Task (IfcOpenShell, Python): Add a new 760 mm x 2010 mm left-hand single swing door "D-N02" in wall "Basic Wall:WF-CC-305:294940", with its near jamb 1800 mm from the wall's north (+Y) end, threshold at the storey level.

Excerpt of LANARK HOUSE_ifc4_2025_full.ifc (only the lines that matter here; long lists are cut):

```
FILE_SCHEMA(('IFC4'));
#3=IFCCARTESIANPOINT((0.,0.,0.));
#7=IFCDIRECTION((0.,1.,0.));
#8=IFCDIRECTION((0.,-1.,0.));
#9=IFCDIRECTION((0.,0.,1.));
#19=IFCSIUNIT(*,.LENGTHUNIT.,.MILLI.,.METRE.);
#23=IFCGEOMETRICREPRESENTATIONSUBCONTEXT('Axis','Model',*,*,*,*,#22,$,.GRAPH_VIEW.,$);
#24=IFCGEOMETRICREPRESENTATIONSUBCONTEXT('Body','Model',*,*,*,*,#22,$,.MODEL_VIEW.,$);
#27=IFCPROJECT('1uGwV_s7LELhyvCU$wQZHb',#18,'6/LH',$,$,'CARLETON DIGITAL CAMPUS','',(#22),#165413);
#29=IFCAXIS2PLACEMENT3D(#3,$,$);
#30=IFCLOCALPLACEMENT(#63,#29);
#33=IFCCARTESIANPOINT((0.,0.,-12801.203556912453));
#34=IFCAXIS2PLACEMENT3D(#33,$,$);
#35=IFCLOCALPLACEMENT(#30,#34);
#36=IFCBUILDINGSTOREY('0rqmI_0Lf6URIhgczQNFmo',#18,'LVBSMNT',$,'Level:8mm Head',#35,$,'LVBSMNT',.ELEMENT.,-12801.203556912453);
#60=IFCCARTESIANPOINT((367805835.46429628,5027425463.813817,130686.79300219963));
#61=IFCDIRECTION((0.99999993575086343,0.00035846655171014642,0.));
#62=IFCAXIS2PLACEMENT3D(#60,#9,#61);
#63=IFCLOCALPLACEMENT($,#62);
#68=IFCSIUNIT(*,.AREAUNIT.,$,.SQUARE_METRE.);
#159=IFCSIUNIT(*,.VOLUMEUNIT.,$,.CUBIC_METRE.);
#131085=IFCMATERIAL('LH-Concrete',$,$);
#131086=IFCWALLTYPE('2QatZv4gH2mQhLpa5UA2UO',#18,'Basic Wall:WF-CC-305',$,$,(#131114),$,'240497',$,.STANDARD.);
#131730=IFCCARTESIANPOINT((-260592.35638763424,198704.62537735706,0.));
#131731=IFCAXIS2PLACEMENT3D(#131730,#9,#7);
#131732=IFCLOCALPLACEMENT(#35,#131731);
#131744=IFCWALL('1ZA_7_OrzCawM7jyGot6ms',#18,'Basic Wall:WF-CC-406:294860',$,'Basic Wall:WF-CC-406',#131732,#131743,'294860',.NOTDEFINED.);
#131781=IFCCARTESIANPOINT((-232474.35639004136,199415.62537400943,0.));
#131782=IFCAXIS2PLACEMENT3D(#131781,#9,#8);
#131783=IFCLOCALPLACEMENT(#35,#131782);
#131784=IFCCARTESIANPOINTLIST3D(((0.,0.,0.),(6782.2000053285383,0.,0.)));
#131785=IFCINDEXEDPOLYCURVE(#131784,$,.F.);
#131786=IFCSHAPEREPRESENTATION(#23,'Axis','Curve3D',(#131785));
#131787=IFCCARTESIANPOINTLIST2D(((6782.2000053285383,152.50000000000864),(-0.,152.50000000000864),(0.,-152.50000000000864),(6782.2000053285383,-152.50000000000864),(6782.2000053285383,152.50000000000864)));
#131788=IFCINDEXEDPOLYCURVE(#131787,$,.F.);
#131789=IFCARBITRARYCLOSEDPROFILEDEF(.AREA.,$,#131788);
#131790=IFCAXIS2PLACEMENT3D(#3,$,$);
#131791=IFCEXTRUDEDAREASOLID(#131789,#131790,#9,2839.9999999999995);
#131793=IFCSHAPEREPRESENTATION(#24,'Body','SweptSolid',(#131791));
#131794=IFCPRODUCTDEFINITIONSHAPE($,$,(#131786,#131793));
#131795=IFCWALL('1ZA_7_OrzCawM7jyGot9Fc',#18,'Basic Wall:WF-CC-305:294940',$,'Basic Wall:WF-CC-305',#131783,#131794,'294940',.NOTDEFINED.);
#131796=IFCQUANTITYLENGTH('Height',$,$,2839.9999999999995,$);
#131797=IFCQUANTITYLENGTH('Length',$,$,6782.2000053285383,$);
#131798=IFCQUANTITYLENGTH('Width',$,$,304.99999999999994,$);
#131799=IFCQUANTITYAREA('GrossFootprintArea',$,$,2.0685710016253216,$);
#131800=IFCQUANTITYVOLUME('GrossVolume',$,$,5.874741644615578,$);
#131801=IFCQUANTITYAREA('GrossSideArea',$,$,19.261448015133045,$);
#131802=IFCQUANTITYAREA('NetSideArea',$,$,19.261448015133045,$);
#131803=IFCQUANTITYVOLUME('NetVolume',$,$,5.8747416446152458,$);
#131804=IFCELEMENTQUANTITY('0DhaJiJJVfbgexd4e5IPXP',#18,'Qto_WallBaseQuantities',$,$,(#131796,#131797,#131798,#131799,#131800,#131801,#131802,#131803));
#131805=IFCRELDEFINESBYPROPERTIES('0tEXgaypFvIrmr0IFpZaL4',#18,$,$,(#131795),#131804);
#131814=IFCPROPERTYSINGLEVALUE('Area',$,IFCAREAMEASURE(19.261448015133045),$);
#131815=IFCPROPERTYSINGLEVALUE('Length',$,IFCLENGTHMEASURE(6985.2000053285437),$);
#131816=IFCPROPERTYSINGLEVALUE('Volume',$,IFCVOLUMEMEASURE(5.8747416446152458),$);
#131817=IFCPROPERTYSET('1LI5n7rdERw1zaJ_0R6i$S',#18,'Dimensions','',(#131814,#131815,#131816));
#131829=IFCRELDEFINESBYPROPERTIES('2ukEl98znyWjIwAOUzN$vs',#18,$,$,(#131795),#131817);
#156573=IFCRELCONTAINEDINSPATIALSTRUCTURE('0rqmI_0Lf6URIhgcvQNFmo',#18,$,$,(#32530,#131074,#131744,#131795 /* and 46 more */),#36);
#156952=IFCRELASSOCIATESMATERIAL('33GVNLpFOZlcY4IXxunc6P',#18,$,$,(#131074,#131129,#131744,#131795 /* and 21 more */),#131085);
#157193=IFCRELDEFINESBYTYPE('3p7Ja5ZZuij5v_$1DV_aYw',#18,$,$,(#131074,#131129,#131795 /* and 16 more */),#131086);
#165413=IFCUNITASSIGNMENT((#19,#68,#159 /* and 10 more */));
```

```python
import numpy as np
import ifcopenshell
import ifcopenshell.api.feature
import ifcopenshell.api.geometry
import ifcopenshell.api.pset
import ifcopenshell.api.root
import ifcopenshell.api.spatial
import ifcopenshell.geom
import ifcopenshell.util.element
import ifcopenshell.util.placement
import ifcopenshell.util.representation
import ifcopenshell.util.shape
import ifcopenshell.util.unit

model = ifcopenshell.open("LANARK HOUSE_ifc4_2025_full.ifc")
unit_scale = ifcopenshell.util.unit.calculate_unit_scale(model)
area_scale = ifcopenshell.util.unit.calculate_unit_scale(model, "AREAUNIT")
volume_scale = ifcopenshell.util.unit.calculate_unit_scale(model, "VOLUMEUNIT")
settings = ifcopenshell.geom.settings()


def volume(element):
    """Net volume in cubic metres, openings subtracted."""
    shape = ifcopenshell.geom.create_shape(settings, element)
    return ifcopenshell.util.shape.get_volume(shape.geometry)


wall = model.by_id(131795)
storey = ifcopenshell.util.element.get_container(wall, ifc_class="IfcBuildingStorey")
context = ifcopenshell.util.representation.get_context(model, "Model", "Body", "MODEL_VIEW")
before = volume(wall)

width, height, from_end, sill = 0.76, 2.01, 1.8, 0.0  # metres

# The wall runs along its own X axis, and the end named is its -X end.
wall_shape = ifcopenshell.geom.create_shape(settings, wall)
x, y, z = ifcopenshell.util.shape.get_vertices(wall_shape.geometry).T
start = x.min() + from_end
face, thickness = float(y.min()), float(y.max() - y.min())
wall_matrix = ifcopenshell.util.placement.get_local_placement(wall.ObjectPlacement)
level = ifcopenshell.util.placement.get_local_placement(storey.ObjectPlacement)[2, 3]


def in_wall(x, y):
    """Placement at x, y metres in the wall's axes, at sill height."""
    matrix = wall_matrix.copy()
    matrix[:, 3] = wall_matrix @ np.array([x / unit_scale, y / unit_scale, 0.0, 1.0])
    matrix[2, 3] = level + sill / unit_scale
    return matrix


# Opening: a box that overshoots both wall faces by 50 mm.
opening = ifcopenshell.api.root.create_entity(model, ifc_class="IfcOpeningElement", predefined_type="OPENING")
box = ifcopenshell.api.geometry.add_wall_representation(
    model, context=context, length=width, height=height, thickness=thickness + 0.1
)
ifcopenshell.api.geometry.assign_representation(model, product=opening, representation=box)
ifcopenshell.api.geometry.edit_object_placement(model, product=opening, matrix=in_wall(start, face - 0.05), is_si=False)
ifcopenshell.api.feature.add_feature(model, feature=opening, element=wall)

door = ifcopenshell.api.root.create_entity(model, ifc_class="IfcDoor", name="D-N02", predefined_type="DOOR")
door.OverallWidth, door.OverallHeight = width / unit_scale, height / unit_scale
door.OperationType = "SINGLE_SWING_LEFT"
body = ifcopenshell.api.geometry.add_door_representation(
    model,
    context=context,
    overall_width=door.OverallWidth,
    overall_height=door.OverallHeight,
    operation_type="SINGLE_SWING_LEFT",
    lining_properties={"LiningDepth": thickness / unit_scale, "ThresholdDepth": thickness / unit_scale},
)
ifcopenshell.api.geometry.assign_representation(model, product=door, representation=body)
ifcopenshell.api.spatial.assign_container(model, products=[door], relating_structure=storey)
ifcopenshell.api.feature.add_filling(model, opening=opening, element=door)

# The lining spans the wall, so the door starts at the wall face.
ifcopenshell.api.geometry.edit_object_placement(model, product=door, matrix=in_wall(start, face), is_si=False)

after = volume(wall)

# Update the wall's stored quantities.
qto = model.by_id(ifcopenshell.util.element.get_pset(wall, "Qto_WallBaseQuantities", should_inherit=False)["id"])
ifcopenshell.api.pset.edit_qto(model, qto=qto, properties={
    "NetSideArea": after / thickness / area_scale,
    "NetVolume": after / volume_scale,
})
pset = model.by_id(ifcopenshell.util.element.get_pset(wall, "Dimensions", should_inherit=False)["id"])
ifcopenshell.api.pset.edit_pset(model, pset=pset, properties={
    "Area": model.create_entity("IfcAreaMeasure", after / thickness / area_scale),
    "Volume": model.create_entity("IfcVolumeMeasure", after / volume_scale),
})

print(f"wall volume {before:.3f} -> {after:.3f} m3")

model.write("LANARK HOUSE_ifc4_2025_full-out.ifc")
```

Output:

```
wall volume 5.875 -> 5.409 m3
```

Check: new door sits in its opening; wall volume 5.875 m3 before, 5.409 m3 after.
